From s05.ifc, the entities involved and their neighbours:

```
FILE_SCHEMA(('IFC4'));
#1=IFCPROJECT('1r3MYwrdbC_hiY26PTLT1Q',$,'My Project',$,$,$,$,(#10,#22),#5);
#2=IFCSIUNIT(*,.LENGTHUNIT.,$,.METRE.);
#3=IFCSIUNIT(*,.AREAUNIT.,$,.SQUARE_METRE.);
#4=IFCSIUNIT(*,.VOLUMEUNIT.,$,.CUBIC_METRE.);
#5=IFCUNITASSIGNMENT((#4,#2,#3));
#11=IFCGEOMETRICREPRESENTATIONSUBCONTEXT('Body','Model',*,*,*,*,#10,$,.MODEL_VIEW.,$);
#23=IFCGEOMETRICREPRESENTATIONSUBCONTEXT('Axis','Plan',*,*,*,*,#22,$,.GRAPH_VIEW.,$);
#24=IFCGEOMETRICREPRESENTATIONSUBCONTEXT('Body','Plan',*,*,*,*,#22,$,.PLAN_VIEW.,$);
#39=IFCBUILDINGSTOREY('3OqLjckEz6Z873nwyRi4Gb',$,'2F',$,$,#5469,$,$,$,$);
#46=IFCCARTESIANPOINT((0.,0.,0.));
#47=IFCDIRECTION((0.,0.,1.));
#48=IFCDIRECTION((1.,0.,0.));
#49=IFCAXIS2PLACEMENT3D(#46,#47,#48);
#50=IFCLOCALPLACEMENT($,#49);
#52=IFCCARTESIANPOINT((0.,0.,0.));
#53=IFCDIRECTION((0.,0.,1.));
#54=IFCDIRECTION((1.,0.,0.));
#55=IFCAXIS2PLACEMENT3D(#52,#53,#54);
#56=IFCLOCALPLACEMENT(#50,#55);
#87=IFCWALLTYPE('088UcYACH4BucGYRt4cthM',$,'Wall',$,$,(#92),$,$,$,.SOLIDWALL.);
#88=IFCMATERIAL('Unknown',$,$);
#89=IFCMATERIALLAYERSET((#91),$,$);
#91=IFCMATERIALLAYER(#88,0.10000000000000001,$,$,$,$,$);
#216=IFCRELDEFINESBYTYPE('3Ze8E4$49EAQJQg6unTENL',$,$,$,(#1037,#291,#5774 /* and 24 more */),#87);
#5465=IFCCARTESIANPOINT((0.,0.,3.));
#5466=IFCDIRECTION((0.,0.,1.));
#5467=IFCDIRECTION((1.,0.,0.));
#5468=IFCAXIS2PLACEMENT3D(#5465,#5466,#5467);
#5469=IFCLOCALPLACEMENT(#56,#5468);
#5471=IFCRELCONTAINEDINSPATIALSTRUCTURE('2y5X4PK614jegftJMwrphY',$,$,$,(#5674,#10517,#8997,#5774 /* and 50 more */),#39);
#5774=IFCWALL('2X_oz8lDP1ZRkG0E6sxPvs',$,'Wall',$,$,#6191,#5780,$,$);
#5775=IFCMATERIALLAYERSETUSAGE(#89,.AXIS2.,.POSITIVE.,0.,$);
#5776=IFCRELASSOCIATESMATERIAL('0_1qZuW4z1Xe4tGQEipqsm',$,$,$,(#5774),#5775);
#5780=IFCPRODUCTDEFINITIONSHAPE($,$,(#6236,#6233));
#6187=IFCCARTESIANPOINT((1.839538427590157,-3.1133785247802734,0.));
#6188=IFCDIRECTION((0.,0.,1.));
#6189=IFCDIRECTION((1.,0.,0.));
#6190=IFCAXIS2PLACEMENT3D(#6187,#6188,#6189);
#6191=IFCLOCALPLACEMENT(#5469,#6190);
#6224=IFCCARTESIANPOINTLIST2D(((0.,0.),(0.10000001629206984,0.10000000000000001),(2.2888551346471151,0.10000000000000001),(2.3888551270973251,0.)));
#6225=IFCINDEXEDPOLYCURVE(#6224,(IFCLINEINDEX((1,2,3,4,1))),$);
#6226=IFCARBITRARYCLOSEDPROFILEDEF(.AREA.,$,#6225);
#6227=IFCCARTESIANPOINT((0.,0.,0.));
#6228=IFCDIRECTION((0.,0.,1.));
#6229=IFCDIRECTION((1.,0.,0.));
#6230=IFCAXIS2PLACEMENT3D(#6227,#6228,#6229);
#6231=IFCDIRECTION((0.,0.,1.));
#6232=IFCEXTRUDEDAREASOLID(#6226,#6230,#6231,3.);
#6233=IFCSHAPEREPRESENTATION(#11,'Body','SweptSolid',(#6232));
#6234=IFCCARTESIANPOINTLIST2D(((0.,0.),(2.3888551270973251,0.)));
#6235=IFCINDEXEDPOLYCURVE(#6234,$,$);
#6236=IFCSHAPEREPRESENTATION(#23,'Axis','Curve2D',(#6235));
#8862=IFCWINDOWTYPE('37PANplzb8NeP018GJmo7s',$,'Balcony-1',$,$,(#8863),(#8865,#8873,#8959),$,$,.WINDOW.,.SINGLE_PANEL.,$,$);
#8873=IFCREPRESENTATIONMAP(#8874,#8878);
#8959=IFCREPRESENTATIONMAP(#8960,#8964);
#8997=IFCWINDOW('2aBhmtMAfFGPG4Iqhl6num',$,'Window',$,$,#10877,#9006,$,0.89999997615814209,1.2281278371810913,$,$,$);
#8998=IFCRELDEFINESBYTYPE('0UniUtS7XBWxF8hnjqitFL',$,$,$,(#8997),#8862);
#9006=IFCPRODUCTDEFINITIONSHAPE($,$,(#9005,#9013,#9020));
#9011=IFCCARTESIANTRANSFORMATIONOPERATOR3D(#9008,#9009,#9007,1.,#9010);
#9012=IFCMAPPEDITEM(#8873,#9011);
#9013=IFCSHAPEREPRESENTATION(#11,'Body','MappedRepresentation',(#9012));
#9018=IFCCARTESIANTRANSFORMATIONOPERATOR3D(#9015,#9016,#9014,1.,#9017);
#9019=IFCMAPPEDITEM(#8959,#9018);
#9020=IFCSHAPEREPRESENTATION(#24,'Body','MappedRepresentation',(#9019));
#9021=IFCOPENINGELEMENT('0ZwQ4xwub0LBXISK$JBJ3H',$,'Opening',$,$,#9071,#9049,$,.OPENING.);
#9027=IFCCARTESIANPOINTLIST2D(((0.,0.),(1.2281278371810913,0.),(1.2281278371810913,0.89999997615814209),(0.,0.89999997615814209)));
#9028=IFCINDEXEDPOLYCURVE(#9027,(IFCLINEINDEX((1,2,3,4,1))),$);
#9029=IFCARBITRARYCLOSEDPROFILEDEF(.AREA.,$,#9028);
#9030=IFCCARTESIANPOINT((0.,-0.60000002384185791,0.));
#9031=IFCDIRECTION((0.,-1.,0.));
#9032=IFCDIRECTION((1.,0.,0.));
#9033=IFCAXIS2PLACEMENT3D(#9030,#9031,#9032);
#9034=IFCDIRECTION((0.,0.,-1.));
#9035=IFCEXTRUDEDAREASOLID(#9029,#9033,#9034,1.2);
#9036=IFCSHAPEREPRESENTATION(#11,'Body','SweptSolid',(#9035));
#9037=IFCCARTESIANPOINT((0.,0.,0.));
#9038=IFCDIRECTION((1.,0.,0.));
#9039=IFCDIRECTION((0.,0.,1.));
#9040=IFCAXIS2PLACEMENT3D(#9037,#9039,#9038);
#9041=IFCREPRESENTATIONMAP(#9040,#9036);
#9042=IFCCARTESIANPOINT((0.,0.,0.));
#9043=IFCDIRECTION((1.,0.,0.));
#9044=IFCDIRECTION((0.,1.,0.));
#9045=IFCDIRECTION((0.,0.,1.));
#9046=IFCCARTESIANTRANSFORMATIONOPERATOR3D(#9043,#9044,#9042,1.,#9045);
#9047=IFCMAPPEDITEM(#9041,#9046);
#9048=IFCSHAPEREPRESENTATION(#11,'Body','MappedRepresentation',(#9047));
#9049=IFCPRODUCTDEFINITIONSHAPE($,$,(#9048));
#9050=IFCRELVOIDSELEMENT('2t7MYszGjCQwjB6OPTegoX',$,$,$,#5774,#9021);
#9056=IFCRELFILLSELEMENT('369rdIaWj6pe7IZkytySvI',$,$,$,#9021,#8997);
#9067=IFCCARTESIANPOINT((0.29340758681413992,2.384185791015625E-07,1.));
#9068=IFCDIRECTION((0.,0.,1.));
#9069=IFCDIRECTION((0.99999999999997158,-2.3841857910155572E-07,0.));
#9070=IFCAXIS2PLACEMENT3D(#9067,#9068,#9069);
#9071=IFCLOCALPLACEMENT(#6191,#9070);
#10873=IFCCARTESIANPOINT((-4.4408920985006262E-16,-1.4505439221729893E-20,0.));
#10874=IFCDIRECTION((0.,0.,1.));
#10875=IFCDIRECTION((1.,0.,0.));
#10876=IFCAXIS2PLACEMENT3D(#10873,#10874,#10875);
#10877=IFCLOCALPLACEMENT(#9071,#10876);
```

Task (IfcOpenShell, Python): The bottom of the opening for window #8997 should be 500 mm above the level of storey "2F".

```python
import numpy as np
import ifcopenshell
import ifcopenshell.api.geometry
import ifcopenshell.geom
import ifcopenshell.util.element
import ifcopenshell.util.placement
import ifcopenshell.util.shape
import ifcopenshell.util.unit

model = ifcopenshell.open("s05.ifc")
unit_scale = ifcopenshell.util.unit.calculate_unit_scale(model)

window = model.by_guid("2aBhmtMAfFGPG4Iqhl6num")
opening = window.FillsVoids[0].RelatingOpeningElement
storey = ifcopenshell.util.element.get_container(window, ifc_class="IfcBuildingStorey")
level = ifcopenshell.util.placement.get_local_placement(storey.ObjectPlacement)[2, 3]

# The opening's origin need not be at the sill, so measure its lowest point.
shape = ifcopenshell.geom.create_shape(ifcopenshell.geom.settings(), opening)
bottom = ifcopenshell.util.shape.get_shape_bottom_elevation(shape, shape.geometry) / unit_scale
dz = level + 0.5 / unit_scale - bottom

shift = np.array([0.0, 0.0, dz])
# The window is placed relative to its opening, so it follows when the opening moves.
matrix = ifcopenshell.util.placement.get_local_placement(opening.ObjectPlacement)
matrix[:3, 3] += shift
ifcopenshell.api.geometry.edit_object_placement(
    model, product=opening, matrix=matrix, is_si=False, should_transform_children=True
)

print(f"moved by {dz * unit_scale:+.3f} m")

model.write("s05-out.ifc")
```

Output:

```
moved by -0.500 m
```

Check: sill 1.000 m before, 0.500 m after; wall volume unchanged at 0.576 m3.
